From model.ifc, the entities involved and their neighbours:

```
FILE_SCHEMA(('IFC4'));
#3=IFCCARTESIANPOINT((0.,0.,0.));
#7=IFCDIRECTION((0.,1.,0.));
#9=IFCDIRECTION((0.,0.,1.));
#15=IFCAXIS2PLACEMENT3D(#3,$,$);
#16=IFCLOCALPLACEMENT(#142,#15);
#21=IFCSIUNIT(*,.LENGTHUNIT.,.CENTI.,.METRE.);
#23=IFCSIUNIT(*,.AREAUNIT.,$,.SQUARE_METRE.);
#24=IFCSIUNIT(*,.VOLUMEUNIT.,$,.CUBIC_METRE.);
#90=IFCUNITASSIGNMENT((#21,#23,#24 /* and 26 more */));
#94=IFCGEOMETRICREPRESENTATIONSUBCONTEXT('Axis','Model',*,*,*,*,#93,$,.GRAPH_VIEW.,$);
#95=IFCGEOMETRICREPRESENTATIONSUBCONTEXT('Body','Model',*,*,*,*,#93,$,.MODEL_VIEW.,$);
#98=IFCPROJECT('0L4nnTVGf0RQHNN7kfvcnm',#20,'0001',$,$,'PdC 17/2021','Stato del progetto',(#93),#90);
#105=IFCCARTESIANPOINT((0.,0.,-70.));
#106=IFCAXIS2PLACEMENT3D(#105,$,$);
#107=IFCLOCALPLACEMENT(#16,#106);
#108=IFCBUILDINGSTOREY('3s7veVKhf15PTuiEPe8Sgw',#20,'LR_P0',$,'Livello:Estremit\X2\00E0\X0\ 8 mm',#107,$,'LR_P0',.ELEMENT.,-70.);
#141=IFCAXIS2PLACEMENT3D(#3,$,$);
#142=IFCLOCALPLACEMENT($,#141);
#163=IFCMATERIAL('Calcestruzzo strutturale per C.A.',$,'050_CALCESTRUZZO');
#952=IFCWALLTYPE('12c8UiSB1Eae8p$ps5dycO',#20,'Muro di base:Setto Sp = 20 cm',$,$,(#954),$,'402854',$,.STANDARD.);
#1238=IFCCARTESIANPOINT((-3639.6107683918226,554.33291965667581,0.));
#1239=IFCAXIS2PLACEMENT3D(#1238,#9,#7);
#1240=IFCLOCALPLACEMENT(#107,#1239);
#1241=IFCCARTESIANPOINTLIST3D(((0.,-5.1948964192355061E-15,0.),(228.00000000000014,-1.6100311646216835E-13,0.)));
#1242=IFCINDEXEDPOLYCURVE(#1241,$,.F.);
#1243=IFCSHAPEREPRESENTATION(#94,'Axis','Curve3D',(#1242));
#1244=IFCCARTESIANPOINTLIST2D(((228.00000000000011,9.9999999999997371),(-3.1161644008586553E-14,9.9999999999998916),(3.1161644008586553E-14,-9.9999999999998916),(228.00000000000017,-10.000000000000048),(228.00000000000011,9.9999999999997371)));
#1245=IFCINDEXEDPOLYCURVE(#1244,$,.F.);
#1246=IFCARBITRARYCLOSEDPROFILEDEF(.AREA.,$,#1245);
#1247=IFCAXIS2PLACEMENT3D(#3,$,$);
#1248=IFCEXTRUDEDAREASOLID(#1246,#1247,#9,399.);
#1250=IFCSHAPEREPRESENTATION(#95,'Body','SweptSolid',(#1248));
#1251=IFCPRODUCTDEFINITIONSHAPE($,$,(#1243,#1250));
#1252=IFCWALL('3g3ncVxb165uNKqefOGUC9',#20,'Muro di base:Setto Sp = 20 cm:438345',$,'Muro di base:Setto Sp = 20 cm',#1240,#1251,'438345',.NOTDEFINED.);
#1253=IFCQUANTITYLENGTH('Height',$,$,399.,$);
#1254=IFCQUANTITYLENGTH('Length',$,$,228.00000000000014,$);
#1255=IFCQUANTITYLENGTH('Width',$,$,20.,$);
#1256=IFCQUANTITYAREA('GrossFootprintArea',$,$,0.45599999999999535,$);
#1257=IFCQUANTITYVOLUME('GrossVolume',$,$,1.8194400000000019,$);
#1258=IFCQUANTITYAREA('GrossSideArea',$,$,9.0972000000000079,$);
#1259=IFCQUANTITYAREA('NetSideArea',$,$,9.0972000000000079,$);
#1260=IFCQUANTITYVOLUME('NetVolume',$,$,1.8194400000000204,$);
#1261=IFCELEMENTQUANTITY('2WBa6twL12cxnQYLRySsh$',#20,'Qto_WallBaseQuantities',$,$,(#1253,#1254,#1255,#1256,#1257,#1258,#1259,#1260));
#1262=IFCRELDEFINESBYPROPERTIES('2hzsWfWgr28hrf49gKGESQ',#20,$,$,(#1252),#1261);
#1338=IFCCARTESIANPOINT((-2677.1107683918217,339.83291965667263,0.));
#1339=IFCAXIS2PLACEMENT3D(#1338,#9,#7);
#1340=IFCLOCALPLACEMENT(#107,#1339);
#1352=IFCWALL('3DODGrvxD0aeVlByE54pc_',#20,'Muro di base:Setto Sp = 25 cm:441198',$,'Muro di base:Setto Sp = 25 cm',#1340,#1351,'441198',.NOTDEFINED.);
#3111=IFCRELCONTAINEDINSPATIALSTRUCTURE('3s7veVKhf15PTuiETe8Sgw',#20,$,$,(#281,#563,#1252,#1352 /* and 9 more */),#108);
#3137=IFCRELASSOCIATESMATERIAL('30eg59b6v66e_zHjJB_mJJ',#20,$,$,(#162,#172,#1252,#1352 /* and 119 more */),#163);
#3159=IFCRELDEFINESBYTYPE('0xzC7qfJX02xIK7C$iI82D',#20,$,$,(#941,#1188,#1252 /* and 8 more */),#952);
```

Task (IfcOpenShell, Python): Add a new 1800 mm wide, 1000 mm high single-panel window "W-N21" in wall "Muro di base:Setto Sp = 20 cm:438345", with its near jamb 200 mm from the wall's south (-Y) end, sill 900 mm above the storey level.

```python
import numpy as np
import ifcopenshell
import ifcopenshell.api.feature
import ifcopenshell.api.geometry
import ifcopenshell.api.pset
import ifcopenshell.api.root
import ifcopenshell.api.spatial
import ifcopenshell.geom
import ifcopenshell.util.element
import ifcopenshell.util.placement
import ifcopenshell.util.representation
import ifcopenshell.util.shape
import ifcopenshell.util.unit

model = ifcopenshell.open("model.ifc")
unit_scale = ifcopenshell.util.unit.calculate_unit_scale(model)
area_scale = ifcopenshell.util.unit.calculate_unit_scale(model, "AREAUNIT")
volume_scale = ifcopenshell.util.unit.calculate_unit_scale(model, "VOLUMEUNIT")
settings = ifcopenshell.geom.settings()


def volume(element):
    """Net volume in cubic metres, openings subtracted."""
    shape = ifcopenshell.geom.create_shape(settings, element)
    return ifcopenshell.util.shape.get_volume(shape.geometry)


wall = model.by_id(1252)
storey = ifcopenshell.util.element.get_container(wall, ifc_class="IfcBuildingStorey")
context = ifcopenshell.util.representation.get_context(model, "Model", "Body", "MODEL_VIEW")
before = volume(wall)

width, height, from_end, sill = 1.8, 1, 0.2, 0.9  # metres

# The wall runs along its own X axis, and the end named is its -X end.
wall_shape = ifcopenshell.geom.create_shape(settings, wall)
x, y, z = ifcopenshell.util.shape.get_vertices(wall_shape.geometry).T
start = x.min() + from_end
face, thickness = float(y.min()), float(y.max() - y.min())
wall_matrix = ifcopenshell.util.placement.get_local_placement(wall.ObjectPlacement)
level = ifcopenshell.util.placement.get_local_placement(storey.ObjectPlacement)[2, 3]


def in_wall(x, y):
    """Placement at x, y metres in the wall's axes, at sill height."""
    matrix = wall_matrix.copy()
    matrix[:, 3] = wall_matrix @ np.array([x / unit_scale, y / unit_scale, 0.0, 1.0])
    matrix[2, 3] = level + sill / unit_scale
    return matrix


# Opening: a box that overshoots both wall faces by 50 mm.
opening = ifcopenshell.api.root.create_entity(model, ifc_class="IfcOpeningElement", predefined_type="OPENING")
box = ifcopenshell.api.geometry.add_wall_representation(
    model, context=context, length=width, height=height, thickness=thickness + 0.1
)
ifcopenshell.api.geometry.assign_representation(model, product=opening, representation=box)
ifcopenshell.api.geometry.edit_object_placement(model, product=opening, matrix=in_wall(start, face - 0.05), is_si=False)
ifcopenshell.api.feature.add_feature(model, feature=opening, element=wall)

window = ifcopenshell.api.root.create_entity(model, ifc_class="IfcWindow", name="W-N21", predefined_type="WINDOW")
window.OverallWidth, window.OverallHeight = width / unit_scale, height / unit_scale
window.PartitioningType = "SINGLE_PANEL"
body = ifcopenshell.api.geometry.add_window_representation(
    model,
    context=context,
    overall_width=window.OverallWidth,
    overall_height=window.OverallHeight,
    partition_type="SINGLE_PANEL",
)
ifcopenshell.api.geometry.assign_representation(model, product=window, representation=body)
ifcopenshell.api.spatial.assign_container(model, products=[window], relating_structure=storey)
ifcopenshell.api.feature.add_filling(model, opening=opening, element=window)

# Centre the window in the wall's thickness.
ifcopenshell.api.geometry.edit_object_placement(model, product=window, matrix=in_wall(start, face), is_si=False)
window_shape = ifcopenshell.geom.create_shape(settings, window)
depth = ifcopenshell.util.shape.get_vertices(window_shape.geometry)[:, 1]
offset = face + thickness / 2 - (depth.min() + depth.max()) / 2
ifcopenshell.api.geometry.edit_object_placement(model, product=window, matrix=in_wall(start, offset), is_si=False)

after = volume(wall)

# Update the wall's stored quantities.
qto = model.by_id(ifcopenshell.util.element.get_pset(wall, "Qto_WallBaseQuantities", should_inherit=False)["id"])
ifcopenshell.api.pset.edit_qto(model, qto=qto, properties={
    "NetSideArea": after / thickness / area_scale,
    "NetVolume": after / volume_scale,
})

print(f"wall volume {before:.3f} -> {after:.3f} m3")

model.write("model-out.ifc")
```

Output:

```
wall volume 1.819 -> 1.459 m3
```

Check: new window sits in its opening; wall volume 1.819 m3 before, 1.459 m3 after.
